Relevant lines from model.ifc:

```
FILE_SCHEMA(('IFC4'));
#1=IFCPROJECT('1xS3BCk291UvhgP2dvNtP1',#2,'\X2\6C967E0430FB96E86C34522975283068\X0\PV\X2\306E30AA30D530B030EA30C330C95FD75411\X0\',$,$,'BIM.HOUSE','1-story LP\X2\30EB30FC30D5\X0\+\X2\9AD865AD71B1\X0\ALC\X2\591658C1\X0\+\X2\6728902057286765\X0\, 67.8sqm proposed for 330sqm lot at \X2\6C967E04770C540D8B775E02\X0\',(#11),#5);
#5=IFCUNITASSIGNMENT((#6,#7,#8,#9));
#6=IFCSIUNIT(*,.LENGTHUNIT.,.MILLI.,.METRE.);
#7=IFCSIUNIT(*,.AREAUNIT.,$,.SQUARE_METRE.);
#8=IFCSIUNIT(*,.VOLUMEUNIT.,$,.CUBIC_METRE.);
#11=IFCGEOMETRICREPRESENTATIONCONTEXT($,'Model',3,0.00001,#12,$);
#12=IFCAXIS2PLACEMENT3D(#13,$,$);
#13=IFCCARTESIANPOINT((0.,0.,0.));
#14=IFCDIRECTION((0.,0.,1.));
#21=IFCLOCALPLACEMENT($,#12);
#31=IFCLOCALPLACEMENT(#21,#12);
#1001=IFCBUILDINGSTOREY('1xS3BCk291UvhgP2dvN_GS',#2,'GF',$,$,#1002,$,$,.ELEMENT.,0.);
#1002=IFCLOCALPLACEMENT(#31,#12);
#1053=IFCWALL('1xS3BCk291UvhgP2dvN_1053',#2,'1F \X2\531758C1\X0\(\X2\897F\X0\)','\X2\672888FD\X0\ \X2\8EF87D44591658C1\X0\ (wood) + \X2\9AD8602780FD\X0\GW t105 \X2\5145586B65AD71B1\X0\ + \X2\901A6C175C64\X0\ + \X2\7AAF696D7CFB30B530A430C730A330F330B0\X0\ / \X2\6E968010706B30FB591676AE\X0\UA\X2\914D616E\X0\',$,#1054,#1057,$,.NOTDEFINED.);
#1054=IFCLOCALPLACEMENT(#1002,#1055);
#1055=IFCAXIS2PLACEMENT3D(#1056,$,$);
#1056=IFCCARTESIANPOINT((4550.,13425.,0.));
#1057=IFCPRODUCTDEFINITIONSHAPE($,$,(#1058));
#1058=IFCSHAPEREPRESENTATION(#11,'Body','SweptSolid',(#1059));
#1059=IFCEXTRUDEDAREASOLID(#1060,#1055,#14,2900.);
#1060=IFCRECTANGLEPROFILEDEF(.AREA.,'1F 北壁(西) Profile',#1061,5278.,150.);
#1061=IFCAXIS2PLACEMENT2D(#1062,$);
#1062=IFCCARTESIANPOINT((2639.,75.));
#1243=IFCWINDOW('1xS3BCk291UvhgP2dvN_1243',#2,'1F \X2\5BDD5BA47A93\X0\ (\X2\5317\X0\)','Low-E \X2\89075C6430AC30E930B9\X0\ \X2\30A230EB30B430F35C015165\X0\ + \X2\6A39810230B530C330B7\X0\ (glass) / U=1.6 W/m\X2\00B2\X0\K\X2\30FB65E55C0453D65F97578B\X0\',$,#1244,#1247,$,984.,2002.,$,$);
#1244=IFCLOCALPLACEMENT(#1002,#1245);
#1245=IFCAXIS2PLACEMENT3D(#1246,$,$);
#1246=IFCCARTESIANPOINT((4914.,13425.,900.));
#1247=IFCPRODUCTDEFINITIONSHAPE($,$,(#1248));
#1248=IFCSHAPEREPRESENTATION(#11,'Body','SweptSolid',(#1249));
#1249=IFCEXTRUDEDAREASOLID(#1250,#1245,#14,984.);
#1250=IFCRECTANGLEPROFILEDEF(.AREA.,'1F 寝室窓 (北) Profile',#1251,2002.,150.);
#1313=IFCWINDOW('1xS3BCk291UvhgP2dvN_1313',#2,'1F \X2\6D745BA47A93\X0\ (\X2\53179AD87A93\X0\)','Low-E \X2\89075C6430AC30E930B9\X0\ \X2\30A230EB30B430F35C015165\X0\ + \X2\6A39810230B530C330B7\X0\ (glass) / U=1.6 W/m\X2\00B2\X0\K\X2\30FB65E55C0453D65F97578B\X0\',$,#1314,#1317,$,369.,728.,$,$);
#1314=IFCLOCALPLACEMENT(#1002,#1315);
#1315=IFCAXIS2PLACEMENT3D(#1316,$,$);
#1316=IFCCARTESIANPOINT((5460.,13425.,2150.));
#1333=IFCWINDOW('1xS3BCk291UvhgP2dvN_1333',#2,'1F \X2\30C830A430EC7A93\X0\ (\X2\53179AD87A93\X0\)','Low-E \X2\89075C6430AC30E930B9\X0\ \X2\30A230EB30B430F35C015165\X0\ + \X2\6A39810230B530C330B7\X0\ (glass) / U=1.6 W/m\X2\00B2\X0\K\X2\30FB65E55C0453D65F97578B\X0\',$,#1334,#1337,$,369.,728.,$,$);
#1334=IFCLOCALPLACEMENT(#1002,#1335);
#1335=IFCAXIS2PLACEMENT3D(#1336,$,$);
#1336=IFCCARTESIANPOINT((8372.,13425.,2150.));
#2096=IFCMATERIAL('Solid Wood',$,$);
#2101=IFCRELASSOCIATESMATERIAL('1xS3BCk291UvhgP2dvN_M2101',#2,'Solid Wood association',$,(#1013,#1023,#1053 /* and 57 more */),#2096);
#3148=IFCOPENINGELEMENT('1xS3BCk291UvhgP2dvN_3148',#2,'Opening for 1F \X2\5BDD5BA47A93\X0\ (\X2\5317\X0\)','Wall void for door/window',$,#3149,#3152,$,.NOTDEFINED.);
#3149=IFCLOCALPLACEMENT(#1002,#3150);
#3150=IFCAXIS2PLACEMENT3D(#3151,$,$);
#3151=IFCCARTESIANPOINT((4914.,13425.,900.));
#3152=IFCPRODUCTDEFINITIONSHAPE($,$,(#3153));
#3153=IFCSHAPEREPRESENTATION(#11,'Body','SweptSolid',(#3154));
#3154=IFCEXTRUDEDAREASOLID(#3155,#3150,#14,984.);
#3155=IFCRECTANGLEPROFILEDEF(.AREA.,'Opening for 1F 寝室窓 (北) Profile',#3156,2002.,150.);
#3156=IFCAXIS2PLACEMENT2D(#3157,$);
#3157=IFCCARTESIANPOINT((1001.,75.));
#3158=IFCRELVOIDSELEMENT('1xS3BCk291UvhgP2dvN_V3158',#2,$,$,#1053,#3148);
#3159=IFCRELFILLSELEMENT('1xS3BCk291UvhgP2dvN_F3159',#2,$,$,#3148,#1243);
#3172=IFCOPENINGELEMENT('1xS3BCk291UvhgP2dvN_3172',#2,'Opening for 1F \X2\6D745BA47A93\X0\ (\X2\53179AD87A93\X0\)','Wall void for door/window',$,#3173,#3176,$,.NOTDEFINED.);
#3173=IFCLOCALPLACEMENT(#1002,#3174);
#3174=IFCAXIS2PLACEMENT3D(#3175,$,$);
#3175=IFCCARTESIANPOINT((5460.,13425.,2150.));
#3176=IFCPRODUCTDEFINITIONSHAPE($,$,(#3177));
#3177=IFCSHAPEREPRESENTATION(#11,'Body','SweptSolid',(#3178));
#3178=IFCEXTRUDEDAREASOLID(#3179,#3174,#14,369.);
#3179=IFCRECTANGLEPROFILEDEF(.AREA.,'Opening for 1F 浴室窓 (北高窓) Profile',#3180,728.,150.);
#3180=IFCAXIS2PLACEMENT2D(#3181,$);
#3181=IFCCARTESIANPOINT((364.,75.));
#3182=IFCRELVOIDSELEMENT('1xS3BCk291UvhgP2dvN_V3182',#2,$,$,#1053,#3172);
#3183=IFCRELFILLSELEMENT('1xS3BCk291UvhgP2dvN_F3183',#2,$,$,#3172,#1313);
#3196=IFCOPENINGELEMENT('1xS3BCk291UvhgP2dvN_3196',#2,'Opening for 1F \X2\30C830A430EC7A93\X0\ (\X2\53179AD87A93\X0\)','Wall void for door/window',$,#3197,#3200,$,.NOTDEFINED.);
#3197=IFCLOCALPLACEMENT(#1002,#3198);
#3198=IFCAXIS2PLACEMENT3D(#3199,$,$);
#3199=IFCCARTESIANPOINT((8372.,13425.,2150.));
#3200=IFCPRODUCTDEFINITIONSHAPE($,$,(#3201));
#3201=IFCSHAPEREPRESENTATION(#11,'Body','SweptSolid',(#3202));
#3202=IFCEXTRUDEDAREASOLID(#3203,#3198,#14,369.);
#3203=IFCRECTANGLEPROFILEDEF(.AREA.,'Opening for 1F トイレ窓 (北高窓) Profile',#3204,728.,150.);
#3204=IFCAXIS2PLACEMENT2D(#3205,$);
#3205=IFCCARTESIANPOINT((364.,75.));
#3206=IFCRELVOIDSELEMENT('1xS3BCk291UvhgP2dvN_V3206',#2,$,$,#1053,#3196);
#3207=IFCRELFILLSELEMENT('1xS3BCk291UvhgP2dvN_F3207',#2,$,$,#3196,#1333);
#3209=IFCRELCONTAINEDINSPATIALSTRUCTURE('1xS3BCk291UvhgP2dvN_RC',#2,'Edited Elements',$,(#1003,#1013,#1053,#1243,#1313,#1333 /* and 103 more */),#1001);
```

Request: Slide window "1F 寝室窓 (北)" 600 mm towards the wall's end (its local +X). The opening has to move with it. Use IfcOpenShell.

```python
import ifcopenshell
import ifcopenshell.api.geometry
import ifcopenshell.util.placement
import ifcopenshell.util.unit

model = ifcopenshell.open("model.ifc")
unit_scale = ifcopenshell.util.unit.calculate_unit_scale(model)

window = model.by_guid("1xS3BCk291UvhgP2dvN_1243")
opening = window.FillsVoids[0].RelatingOpeningElement
wall = opening.VoidsElements[0].RelatingBuildingElement

wall_matrix = ifcopenshell.util.placement.get_local_placement(wall.ObjectPlacement)
shift = wall_matrix[:3, 0] * 0.6 / unit_scale
before = ifcopenshell.util.placement.get_local_placement(window.ObjectPlacement)[:3, 3].copy()

# The window is not placed relative to its opening, so move both.
for product in (opening, window):
    matrix = ifcopenshell.util.placement.get_local_placement(product.ObjectPlacement)
    matrix[:3, 3] += shift
    ifcopenshell.api.geometry.edit_object_placement(model, product=product, matrix=matrix, is_si=False)

after = ifcopenshell.util.placement.get_local_placement(window.ObjectPlacement)[:3, 3]
print("window moved by", (after - before).round(3) + 0.0)

model.write("model_rev.ifc")
```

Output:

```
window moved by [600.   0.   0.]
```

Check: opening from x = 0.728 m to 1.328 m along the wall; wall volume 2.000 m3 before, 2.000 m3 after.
